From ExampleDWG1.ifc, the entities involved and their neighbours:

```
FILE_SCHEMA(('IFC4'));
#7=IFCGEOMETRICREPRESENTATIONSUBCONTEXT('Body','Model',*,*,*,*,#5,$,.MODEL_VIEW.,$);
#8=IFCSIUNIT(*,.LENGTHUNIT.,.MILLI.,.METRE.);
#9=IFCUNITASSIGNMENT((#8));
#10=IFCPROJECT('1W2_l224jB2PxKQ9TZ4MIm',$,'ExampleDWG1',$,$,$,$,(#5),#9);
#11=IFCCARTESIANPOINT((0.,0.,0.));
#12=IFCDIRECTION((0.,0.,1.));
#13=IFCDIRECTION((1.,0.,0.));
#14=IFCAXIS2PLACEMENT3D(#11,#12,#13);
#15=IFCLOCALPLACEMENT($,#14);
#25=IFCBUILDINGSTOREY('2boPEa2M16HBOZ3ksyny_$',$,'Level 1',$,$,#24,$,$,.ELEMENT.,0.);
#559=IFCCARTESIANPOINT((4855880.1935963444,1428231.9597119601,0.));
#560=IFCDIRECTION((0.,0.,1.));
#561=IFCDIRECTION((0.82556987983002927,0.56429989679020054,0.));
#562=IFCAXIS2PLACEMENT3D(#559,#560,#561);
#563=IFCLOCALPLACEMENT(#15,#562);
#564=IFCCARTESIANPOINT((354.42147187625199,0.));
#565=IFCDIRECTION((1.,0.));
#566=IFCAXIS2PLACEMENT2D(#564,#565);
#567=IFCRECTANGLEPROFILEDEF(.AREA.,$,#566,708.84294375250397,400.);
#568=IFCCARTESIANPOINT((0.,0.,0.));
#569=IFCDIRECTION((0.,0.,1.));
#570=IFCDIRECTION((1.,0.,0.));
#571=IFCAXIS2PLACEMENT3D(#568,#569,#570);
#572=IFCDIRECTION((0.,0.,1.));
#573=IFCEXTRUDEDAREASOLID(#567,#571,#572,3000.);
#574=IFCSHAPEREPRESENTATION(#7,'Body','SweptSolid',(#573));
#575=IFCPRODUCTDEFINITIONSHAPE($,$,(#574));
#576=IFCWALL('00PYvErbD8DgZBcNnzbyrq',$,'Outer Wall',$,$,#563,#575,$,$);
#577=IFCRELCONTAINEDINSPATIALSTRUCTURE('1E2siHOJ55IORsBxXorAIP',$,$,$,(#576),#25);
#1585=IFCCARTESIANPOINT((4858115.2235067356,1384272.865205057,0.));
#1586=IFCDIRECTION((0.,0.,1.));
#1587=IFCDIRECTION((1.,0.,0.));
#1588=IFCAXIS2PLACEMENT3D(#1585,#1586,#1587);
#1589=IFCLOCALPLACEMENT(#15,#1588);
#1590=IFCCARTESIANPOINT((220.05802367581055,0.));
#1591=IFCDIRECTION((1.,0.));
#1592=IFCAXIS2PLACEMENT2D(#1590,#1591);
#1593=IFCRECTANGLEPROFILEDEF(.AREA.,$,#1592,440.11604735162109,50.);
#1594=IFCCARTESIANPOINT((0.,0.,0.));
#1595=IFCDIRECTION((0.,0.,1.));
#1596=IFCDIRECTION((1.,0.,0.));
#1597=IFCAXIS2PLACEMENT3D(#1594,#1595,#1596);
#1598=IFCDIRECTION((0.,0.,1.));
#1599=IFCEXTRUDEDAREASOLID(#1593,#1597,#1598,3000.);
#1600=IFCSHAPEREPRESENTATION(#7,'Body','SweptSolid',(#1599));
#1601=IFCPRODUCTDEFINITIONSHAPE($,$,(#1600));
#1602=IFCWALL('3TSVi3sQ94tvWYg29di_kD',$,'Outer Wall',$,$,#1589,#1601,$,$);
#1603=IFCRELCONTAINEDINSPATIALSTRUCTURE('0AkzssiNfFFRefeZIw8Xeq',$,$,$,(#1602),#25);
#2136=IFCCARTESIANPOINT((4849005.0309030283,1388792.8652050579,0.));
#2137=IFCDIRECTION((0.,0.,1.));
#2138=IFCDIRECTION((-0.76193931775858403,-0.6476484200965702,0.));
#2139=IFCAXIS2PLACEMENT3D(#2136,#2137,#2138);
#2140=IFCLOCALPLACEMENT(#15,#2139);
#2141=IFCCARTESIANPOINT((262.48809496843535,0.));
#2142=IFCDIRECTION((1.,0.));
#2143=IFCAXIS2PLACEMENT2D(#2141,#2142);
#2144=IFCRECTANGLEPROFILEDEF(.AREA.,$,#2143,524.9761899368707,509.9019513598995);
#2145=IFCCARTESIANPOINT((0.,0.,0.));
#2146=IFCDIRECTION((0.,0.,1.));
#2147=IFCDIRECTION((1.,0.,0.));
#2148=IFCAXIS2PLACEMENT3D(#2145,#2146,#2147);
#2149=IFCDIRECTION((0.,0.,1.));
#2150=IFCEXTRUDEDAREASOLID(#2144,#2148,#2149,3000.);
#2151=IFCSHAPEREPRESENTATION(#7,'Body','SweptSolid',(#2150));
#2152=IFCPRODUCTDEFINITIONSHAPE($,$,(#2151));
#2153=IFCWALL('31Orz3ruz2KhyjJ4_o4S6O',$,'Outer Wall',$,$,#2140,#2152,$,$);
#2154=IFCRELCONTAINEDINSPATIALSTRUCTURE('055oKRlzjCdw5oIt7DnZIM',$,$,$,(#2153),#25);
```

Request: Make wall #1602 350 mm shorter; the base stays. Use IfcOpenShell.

```python
import ifcopenshell
import ifcopenshell.geom
import ifcopenshell.util.representation
import ifcopenshell.util.shape
import ifcopenshell.util.unit

model = ifcopenshell.open("ExampleDWG1.ifc")
unit_scale = ifcopenshell.util.unit.calculate_unit_scale(model)
settings = ifcopenshell.geom.settings()


def volume(element):
    """Net volume in cubic metres, openings subtracted."""
    shape = ifcopenshell.geom.create_shape(settings, element)
    return ifcopenshell.util.shape.get_volume(shape.geometry)


wall = model.by_guid("3TSVi3sQ94tvWYg29di_kD")
before = volume(wall)

body = ifcopenshell.util.representation.get_representation(wall, "Model", "Body")
solid = body.Items[0]
old_height = solid.Depth
solid.Depth -= 0.35 / unit_scale
after = volume(wall)

print(f"height {old_height:g} -> {solid.Depth:g}, volume {before:.3f} -> {after:.3f} m3")

model.write("ExampleDWG1_edited.ifc")
```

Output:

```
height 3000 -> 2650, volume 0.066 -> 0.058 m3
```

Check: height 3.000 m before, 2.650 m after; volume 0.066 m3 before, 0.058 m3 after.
